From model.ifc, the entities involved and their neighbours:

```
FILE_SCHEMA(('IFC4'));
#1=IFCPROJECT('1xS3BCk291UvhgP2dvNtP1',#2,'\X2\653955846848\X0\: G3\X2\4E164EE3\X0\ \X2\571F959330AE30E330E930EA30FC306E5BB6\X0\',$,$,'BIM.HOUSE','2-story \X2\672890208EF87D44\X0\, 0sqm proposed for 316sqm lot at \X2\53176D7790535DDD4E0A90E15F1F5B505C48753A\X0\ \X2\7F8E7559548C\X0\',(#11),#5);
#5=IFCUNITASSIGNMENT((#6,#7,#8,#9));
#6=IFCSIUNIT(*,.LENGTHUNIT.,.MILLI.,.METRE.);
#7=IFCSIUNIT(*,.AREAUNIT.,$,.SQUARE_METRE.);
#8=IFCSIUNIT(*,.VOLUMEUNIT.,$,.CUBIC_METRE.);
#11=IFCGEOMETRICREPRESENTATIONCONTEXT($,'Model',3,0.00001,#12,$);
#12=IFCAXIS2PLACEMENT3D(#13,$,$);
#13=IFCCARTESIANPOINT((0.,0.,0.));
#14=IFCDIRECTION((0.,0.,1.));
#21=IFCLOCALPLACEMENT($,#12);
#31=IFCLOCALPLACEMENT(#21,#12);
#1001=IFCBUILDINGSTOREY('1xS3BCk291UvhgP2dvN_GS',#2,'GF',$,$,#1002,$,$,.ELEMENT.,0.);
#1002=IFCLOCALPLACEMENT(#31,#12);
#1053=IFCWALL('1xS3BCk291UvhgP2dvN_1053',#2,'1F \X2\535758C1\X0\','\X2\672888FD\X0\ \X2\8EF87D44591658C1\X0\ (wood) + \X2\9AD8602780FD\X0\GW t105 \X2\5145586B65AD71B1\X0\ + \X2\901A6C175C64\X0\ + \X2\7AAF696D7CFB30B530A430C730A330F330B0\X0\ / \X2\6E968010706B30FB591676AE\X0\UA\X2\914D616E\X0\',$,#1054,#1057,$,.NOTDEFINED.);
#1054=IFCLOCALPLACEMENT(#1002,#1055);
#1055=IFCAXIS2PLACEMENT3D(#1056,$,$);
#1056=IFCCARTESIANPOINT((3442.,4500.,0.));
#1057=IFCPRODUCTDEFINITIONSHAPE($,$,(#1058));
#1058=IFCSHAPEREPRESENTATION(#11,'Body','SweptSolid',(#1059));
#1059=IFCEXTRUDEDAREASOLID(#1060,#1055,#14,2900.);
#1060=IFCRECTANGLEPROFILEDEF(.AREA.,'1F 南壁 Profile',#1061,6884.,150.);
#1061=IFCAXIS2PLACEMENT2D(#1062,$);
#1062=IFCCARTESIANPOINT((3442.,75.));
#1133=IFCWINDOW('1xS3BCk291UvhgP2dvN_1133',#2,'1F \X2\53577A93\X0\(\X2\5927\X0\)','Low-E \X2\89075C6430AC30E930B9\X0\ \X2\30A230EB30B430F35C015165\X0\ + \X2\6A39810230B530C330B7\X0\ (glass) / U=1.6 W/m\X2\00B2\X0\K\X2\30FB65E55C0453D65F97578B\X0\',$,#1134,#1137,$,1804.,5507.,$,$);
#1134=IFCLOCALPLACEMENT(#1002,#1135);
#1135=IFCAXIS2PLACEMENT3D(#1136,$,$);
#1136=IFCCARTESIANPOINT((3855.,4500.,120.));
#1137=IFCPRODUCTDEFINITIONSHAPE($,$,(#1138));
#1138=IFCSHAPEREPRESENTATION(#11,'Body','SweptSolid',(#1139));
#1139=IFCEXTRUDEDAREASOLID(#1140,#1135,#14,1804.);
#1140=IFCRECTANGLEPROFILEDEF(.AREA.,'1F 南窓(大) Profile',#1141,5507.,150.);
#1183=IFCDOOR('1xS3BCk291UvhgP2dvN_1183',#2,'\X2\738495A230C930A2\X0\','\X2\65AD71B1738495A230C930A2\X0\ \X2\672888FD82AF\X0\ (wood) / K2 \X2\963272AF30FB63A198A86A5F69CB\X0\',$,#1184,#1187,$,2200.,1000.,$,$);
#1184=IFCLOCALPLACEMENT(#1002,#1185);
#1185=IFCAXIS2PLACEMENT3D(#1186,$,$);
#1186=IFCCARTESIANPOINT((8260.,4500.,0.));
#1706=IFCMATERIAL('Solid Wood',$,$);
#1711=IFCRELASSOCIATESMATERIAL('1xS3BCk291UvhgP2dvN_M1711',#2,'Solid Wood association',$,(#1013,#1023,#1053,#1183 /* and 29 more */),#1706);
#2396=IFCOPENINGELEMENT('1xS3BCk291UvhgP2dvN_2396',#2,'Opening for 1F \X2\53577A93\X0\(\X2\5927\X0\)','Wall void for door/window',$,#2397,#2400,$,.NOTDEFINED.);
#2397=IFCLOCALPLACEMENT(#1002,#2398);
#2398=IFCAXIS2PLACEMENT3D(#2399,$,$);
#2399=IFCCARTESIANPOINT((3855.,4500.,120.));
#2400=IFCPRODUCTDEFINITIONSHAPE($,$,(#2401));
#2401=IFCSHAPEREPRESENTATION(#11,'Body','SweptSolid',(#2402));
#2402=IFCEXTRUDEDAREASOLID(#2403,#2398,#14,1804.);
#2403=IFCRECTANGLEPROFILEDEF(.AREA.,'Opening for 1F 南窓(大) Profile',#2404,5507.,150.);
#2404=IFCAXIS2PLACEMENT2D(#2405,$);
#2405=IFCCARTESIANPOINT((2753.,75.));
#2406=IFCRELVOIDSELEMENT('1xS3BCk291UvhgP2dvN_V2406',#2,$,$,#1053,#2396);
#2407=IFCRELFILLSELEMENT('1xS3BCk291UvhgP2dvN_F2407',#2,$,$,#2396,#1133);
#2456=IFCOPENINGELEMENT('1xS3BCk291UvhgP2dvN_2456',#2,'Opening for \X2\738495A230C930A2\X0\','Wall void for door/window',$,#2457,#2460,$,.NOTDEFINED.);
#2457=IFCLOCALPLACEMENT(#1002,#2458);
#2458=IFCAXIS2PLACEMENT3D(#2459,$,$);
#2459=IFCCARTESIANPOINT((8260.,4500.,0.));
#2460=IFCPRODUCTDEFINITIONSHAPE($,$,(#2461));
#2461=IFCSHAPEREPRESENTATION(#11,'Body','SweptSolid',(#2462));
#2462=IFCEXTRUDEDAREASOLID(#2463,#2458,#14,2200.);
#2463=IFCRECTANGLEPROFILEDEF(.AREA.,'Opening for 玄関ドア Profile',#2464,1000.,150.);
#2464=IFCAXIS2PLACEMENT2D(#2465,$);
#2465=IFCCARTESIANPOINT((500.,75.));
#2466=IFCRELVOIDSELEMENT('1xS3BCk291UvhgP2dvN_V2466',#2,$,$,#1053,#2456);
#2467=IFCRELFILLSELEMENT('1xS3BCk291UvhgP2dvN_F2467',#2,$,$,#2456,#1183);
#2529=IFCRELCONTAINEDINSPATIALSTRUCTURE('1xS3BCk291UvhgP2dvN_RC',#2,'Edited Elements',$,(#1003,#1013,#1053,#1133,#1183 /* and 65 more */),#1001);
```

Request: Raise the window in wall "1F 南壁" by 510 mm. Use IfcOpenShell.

```python
import numpy as np
import ifcopenshell
import ifcopenshell.api.geometry
import ifcopenshell.util.placement
import ifcopenshell.util.unit

model = ifcopenshell.open("model.ifc")
unit_scale = ifcopenshell.util.unit.calculate_unit_scale(model)

window = model.by_id(1133)
opening = window.FillsVoids[0].RelatingOpeningElement
dz = 0.51 / unit_scale

shift = np.array([0.0, 0.0, dz])
# The window is not placed relative to its opening, so move both.
for product in (opening, window):
    matrix = ifcopenshell.util.placement.get_local_placement(product.ObjectPlacement)
    matrix[:3, 3] += shift
    ifcopenshell.api.geometry.edit_object_placement(model, product=product, matrix=matrix, is_si=False)

print(f"moved by {dz * unit_scale:+.3f} m")

model.write("model_rev.ifc")
```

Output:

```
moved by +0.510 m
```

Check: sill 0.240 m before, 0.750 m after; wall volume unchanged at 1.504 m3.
